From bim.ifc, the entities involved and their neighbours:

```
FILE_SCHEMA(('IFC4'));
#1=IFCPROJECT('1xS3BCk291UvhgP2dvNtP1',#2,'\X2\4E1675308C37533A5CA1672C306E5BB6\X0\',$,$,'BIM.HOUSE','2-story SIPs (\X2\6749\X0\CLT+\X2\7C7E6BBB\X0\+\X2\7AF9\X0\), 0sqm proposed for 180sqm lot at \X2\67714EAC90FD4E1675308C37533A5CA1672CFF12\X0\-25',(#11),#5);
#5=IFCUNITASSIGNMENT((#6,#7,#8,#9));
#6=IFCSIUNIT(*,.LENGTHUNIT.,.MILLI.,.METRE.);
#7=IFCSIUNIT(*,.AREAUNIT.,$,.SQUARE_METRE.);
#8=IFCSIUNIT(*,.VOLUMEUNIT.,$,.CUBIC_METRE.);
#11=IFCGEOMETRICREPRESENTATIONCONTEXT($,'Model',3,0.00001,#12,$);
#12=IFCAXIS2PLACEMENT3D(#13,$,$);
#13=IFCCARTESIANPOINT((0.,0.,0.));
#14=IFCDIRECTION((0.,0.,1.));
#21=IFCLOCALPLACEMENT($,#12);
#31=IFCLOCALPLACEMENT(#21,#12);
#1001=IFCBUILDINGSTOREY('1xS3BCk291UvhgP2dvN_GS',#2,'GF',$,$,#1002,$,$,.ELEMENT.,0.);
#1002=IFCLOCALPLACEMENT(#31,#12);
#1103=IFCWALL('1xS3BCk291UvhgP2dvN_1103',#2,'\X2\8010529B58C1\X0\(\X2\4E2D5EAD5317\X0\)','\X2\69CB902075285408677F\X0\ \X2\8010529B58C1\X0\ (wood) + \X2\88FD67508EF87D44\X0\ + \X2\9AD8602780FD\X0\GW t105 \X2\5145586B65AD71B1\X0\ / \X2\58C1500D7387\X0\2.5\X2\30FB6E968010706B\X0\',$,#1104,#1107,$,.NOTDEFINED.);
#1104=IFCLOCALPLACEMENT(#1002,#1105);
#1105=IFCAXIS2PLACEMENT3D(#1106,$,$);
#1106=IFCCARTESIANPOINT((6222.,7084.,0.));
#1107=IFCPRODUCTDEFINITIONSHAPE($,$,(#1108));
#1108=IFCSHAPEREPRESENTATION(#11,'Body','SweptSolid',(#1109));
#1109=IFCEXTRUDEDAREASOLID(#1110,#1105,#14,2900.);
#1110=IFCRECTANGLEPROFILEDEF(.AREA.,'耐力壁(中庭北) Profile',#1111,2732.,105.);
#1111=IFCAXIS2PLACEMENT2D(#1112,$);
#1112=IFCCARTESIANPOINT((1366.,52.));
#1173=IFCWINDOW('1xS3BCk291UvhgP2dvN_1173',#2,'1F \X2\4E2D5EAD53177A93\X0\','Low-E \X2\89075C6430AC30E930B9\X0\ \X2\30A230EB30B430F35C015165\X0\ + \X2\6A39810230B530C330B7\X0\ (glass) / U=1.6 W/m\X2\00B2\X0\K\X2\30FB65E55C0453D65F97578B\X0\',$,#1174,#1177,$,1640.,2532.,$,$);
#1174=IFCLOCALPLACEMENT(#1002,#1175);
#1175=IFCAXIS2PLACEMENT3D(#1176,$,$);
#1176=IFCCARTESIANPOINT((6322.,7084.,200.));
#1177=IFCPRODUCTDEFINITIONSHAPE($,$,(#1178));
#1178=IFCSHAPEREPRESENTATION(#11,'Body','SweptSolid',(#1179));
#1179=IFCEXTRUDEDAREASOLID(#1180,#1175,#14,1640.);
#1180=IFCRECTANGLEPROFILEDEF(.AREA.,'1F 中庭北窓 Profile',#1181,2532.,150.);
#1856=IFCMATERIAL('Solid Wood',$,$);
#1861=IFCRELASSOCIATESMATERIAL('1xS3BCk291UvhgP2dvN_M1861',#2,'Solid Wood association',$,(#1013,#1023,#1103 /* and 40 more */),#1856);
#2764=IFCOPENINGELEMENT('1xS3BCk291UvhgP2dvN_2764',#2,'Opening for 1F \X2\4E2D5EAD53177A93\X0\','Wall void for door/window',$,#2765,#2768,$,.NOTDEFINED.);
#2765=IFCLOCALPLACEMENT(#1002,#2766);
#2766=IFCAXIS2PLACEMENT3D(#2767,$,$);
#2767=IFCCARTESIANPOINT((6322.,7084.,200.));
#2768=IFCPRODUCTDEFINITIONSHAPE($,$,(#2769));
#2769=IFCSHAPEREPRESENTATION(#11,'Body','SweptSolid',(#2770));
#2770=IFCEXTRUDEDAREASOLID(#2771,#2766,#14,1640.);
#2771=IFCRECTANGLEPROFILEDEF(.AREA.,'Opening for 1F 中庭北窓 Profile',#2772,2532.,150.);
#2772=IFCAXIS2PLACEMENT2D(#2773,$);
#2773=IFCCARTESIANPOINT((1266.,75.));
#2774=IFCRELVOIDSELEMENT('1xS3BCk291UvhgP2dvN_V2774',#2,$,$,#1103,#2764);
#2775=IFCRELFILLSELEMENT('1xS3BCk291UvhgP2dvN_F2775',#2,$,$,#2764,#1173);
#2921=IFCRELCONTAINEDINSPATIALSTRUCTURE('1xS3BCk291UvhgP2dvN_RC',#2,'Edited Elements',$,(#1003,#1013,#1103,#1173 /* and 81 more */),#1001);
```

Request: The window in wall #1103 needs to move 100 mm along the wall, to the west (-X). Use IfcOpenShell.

```python
import ifcopenshell
import ifcopenshell.api.geometry
import ifcopenshell.util.placement
import ifcopenshell.util.unit

model = ifcopenshell.open("bim.ifc")
unit_scale = ifcopenshell.util.unit.calculate_unit_scale(model)

window = model.by_id(1173)
opening = window.FillsVoids[0].RelatingOpeningElement
wall = opening.VoidsElements[0].RelatingBuildingElement

wall_matrix = ifcopenshell.util.placement.get_local_placement(wall.ObjectPlacement)
shift = wall_matrix[:3, 0] * -0.1 / unit_scale
before = ifcopenshell.util.placement.get_local_placement(window.ObjectPlacement)[:3, 3].copy()

# The window is not placed relative to its opening, so move both.
for product in (opening, window):
    matrix = ifcopenshell.util.placement.get_local_placement(product.ObjectPlacement)
    matrix[:3, 3] += shift
    ifcopenshell.api.geometry.edit_object_placement(model, product=product, matrix=matrix, is_si=False)

after = ifcopenshell.util.placement.get_local_placement(window.ObjectPlacement)[:3, 3]
print("window moved by", (after - before).round(3) + 0.0)

model.write("bim_edited.ifc")
```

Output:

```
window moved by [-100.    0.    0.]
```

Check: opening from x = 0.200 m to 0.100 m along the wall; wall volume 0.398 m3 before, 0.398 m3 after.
